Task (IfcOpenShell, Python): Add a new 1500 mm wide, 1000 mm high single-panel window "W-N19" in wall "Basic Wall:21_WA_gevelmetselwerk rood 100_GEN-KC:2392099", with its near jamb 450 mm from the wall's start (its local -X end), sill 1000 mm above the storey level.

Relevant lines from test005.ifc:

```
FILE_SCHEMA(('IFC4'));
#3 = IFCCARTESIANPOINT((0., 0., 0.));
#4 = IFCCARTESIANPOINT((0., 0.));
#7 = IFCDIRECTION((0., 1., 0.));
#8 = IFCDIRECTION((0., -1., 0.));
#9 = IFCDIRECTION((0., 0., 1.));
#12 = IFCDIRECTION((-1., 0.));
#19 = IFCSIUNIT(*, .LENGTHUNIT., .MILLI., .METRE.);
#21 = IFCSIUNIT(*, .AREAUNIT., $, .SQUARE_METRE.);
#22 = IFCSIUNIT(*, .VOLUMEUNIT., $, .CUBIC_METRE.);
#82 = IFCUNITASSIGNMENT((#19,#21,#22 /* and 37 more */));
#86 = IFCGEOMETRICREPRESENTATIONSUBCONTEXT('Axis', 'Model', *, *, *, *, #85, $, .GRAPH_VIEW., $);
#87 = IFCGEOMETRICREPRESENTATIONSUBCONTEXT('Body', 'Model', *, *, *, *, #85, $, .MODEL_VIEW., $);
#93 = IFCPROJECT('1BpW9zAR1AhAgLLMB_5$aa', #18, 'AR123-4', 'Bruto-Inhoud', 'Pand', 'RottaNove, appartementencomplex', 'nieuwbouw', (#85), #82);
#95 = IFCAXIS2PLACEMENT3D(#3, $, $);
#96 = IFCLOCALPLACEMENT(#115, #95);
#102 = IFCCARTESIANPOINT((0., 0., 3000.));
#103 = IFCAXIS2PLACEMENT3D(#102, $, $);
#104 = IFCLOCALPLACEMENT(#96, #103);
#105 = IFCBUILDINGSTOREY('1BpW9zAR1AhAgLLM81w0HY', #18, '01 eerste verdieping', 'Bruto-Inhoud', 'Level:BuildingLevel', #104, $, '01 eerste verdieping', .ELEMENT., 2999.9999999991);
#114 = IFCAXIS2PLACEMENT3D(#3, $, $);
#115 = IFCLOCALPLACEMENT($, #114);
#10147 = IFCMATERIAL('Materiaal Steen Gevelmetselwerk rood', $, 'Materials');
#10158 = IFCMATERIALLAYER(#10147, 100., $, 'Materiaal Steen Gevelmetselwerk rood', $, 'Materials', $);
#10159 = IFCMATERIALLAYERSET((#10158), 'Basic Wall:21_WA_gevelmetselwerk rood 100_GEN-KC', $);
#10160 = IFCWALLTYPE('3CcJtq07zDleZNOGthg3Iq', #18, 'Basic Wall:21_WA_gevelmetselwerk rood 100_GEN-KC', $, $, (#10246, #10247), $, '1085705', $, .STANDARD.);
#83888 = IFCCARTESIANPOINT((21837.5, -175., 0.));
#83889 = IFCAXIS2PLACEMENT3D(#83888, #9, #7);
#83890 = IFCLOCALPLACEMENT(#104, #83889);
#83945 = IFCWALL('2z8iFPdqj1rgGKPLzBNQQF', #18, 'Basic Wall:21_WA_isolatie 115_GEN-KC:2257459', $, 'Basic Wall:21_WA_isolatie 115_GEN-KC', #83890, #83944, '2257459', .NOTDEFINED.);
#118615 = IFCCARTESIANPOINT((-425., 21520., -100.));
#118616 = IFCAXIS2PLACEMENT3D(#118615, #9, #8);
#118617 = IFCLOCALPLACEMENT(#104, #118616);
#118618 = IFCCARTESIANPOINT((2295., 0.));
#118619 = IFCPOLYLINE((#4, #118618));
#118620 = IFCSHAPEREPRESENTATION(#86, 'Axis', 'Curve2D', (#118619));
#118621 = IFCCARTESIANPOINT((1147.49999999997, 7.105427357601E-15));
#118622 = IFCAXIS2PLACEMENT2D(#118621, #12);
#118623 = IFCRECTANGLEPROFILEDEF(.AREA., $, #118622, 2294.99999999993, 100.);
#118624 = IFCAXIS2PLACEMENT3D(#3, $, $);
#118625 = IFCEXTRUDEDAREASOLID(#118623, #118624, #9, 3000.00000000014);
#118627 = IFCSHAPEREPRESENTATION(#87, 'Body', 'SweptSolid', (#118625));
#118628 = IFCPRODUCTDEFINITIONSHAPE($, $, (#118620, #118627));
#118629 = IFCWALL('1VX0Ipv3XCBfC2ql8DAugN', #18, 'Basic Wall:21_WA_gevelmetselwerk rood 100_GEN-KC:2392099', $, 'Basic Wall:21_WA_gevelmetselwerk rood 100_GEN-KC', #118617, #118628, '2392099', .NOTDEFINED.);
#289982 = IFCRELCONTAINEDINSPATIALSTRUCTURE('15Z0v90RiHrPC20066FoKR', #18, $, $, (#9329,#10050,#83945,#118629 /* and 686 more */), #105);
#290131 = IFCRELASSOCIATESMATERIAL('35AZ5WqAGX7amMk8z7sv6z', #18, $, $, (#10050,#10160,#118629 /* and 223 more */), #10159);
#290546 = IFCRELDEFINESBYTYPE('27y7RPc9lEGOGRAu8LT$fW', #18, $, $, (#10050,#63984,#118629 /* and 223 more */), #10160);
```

```python
import numpy as np
import ifcopenshell
import ifcopenshell.api.feature
import ifcopenshell.api.geometry
import ifcopenshell.api.root
import ifcopenshell.api.spatial
import ifcopenshell.geom
import ifcopenshell.util.element
import ifcopenshell.util.placement
import ifcopenshell.util.representation
import ifcopenshell.util.shape
import ifcopenshell.util.unit

model = ifcopenshell.open("test005.ifc")
unit_scale = ifcopenshell.util.unit.calculate_unit_scale(model)
settings = ifcopenshell.geom.settings()


def volume(element):
    """Net volume in cubic metres, openings subtracted."""
    shape = ifcopenshell.geom.create_shape(settings, element)
    return ifcopenshell.util.shape.get_volume(shape.geometry)


wall = model.by_id(118629)
storey = ifcopenshell.util.element.get_container(wall, ifc_class="IfcBuildingStorey")
context = ifcopenshell.util.representation.get_context(model, "Model", "Body", "MODEL_VIEW")
before = volume(wall)

width, height, from_end, sill = 1.5, 1, 0.45, 1  # metres

# The wall runs along its own X axis, and the end named is its -X end.
wall_shape = ifcopenshell.geom.create_shape(settings, wall)
x, y, z = ifcopenshell.util.shape.get_vertices(wall_shape.geometry).T
start = x.min() + from_end
face, thickness = float(y.min()), float(y.max() - y.min())
wall_matrix = ifcopenshell.util.placement.get_local_placement(wall.ObjectPlacement)
level = ifcopenshell.util.placement.get_local_placement(storey.ObjectPlacement)[2, 3]


def in_wall(x, y):
    """Placement at x, y metres in the wall's axes, at sill height."""
    matrix = wall_matrix.copy()
    matrix[:, 3] = wall_matrix @ np.array([x / unit_scale, y / unit_scale, 0.0, 1.0])
    matrix[2, 3] = level + sill / unit_scale
    return matrix


# Opening: a box that overshoots both wall faces by 50 mm.
opening = ifcopenshell.api.root.create_entity(model, ifc_class="IfcOpeningElement", predefined_type="OPENING")
box = ifcopenshell.api.geometry.add_wall_representation(
    model, context=context, length=width, height=height, thickness=thickness + 0.1
)
ifcopenshell.api.geometry.assign_representation(model, product=opening, representation=box)
ifcopenshell.api.geometry.edit_object_placement(model, product=opening, matrix=in_wall(start, face - 0.05), is_si=False)
ifcopenshell.api.feature.add_feature(model, feature=opening, element=wall)

window = ifcopenshell.api.root.create_entity(model, ifc_class="IfcWindow", name="W-N19", predefined_type="WINDOW")
window.OverallWidth, window.OverallHeight = width / unit_scale, height / unit_scale
window.PartitioningType = "SINGLE_PANEL"
body = ifcopenshell.api.geometry.add_window_representation(
    model,
    context=context,
    overall_width=window.OverallWidth,
    overall_height=window.OverallHeight,
    partition_type="SINGLE_PANEL",
)
ifcopenshell.api.geometry.assign_representation(model, product=window, representation=body)
ifcopenshell.api.spatial.assign_container(model, products=[window], relating_structure=storey)
ifcopenshell.api.feature.add_filling(model, opening=opening, element=window)

# Centre the window in the wall's thickness.
ifcopenshell.api.geometry.edit_object_placement(model, product=window, matrix=in_wall(start, face), is_si=False)
window_shape = ifcopenshell.geom.create_shape(settings, window)
depth = ifcopenshell.util.shape.get_vertices(window_shape.geometry)[:, 1]
offset = face + thickness / 2 - (depth.min() + depth.max()) / 2
ifcopenshell.api.geometry.edit_object_placement(model, product=window, matrix=in_wall(start, offset), is_si=False)

after = volume(wall)

print(f"wall volume {before:.3f} -> {after:.3f} m3")

model.write("test005_v2.ifc")
```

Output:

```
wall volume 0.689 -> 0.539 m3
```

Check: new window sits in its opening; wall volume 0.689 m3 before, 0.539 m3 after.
